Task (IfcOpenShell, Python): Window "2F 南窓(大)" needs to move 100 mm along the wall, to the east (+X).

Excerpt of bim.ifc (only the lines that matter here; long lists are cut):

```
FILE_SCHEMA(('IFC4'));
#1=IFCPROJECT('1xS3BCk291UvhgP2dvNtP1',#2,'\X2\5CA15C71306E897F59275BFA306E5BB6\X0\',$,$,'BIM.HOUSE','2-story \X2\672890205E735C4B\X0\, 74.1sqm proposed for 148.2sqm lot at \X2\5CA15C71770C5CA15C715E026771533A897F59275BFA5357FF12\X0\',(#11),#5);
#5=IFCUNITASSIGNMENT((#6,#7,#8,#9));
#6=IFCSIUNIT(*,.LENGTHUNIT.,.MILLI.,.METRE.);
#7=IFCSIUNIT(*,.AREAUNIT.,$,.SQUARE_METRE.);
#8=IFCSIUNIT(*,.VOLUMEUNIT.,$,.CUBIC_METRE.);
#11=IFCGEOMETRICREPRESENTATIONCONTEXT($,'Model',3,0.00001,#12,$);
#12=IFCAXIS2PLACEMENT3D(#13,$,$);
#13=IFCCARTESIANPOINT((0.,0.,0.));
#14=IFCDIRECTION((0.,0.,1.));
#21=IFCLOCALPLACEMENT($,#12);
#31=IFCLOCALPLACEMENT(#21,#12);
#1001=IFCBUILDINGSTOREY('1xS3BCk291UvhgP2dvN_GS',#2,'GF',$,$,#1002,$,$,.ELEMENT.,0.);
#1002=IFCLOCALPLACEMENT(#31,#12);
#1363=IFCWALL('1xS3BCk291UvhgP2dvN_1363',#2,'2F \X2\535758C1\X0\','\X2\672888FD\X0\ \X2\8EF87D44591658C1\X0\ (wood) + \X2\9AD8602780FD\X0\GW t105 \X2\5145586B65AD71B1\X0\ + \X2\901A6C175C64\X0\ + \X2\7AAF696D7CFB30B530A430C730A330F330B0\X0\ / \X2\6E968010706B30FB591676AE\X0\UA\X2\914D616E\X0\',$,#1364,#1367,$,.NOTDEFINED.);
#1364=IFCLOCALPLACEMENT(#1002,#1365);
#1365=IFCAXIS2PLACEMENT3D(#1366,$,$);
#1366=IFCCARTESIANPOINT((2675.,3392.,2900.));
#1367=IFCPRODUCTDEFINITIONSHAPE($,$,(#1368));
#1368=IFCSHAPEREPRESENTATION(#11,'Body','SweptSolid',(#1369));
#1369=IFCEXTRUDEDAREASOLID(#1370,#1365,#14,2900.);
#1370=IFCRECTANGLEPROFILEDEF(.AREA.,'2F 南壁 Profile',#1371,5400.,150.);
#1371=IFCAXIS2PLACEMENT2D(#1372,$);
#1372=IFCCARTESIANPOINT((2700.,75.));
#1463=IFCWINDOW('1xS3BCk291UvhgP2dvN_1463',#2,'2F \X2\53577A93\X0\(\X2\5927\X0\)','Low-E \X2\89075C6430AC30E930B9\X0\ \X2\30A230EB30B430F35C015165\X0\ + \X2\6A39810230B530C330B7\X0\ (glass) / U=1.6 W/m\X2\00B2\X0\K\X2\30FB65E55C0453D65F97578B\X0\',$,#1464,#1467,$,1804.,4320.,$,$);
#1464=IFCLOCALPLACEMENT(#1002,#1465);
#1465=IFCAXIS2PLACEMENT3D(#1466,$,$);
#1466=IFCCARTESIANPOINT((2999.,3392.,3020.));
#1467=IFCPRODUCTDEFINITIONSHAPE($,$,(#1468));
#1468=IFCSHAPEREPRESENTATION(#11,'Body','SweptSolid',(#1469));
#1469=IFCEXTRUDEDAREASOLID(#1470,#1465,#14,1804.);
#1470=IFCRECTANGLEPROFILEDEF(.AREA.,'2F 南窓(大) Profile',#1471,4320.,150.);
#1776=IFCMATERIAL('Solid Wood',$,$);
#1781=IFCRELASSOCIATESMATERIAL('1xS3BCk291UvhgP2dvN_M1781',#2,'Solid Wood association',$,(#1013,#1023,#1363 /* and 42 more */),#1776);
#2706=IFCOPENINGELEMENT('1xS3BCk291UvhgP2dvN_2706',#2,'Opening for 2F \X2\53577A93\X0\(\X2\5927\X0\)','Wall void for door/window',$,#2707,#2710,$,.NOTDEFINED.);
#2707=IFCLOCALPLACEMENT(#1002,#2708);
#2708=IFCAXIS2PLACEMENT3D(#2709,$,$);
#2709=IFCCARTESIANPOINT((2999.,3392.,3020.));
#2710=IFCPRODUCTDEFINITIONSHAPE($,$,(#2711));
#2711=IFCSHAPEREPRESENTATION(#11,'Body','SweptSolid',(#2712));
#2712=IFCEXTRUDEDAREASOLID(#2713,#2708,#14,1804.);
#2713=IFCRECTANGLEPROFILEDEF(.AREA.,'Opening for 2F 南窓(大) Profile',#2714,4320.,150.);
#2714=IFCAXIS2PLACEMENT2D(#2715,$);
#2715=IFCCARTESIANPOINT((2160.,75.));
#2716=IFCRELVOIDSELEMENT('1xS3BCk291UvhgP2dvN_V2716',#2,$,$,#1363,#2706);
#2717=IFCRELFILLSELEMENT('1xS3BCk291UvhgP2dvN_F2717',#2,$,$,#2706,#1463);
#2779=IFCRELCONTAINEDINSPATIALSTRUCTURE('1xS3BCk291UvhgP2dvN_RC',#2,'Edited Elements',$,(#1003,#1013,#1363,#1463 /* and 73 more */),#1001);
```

```python
import ifcopenshell
import ifcopenshell.api.geometry
import ifcopenshell.util.placement

model = ifcopenshell.open("bim.ifc")

window = model.by_guid("1xS3BCk291UvhgP2dvN_1463")
opening = window.FillsVoids[0].RelatingOpeningElement
wall = opening.VoidsElements[0].RelatingBuildingElement

wall_matrix = ifcopenshell.util.placement.get_local_placement(wall.ObjectPlacement)
shift = wall_matrix[:3, 0] * 100.0
before = ifcopenshell.util.placement.get_local_placement(window.ObjectPlacement)[:3, 3].copy()

# The window is not placed relative to its opening, so move both.
for product in (opening, window):
    matrix = ifcopenshell.util.placement.get_local_placement(product.ObjectPlacement)
    matrix[:3, 3] += shift
    ifcopenshell.api.geometry.edit_object_placement(model, product=product, matrix=matrix, is_si=False)

after = ifcopenshell.util.placement.get_local_placement(window.ObjectPlacement)[:3, 3]
print("window moved by", (after - before).round(3) + 0.0)

model.write("bim-out.ifc")
```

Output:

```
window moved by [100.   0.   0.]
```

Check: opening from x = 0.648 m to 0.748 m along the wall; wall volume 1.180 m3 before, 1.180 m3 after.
